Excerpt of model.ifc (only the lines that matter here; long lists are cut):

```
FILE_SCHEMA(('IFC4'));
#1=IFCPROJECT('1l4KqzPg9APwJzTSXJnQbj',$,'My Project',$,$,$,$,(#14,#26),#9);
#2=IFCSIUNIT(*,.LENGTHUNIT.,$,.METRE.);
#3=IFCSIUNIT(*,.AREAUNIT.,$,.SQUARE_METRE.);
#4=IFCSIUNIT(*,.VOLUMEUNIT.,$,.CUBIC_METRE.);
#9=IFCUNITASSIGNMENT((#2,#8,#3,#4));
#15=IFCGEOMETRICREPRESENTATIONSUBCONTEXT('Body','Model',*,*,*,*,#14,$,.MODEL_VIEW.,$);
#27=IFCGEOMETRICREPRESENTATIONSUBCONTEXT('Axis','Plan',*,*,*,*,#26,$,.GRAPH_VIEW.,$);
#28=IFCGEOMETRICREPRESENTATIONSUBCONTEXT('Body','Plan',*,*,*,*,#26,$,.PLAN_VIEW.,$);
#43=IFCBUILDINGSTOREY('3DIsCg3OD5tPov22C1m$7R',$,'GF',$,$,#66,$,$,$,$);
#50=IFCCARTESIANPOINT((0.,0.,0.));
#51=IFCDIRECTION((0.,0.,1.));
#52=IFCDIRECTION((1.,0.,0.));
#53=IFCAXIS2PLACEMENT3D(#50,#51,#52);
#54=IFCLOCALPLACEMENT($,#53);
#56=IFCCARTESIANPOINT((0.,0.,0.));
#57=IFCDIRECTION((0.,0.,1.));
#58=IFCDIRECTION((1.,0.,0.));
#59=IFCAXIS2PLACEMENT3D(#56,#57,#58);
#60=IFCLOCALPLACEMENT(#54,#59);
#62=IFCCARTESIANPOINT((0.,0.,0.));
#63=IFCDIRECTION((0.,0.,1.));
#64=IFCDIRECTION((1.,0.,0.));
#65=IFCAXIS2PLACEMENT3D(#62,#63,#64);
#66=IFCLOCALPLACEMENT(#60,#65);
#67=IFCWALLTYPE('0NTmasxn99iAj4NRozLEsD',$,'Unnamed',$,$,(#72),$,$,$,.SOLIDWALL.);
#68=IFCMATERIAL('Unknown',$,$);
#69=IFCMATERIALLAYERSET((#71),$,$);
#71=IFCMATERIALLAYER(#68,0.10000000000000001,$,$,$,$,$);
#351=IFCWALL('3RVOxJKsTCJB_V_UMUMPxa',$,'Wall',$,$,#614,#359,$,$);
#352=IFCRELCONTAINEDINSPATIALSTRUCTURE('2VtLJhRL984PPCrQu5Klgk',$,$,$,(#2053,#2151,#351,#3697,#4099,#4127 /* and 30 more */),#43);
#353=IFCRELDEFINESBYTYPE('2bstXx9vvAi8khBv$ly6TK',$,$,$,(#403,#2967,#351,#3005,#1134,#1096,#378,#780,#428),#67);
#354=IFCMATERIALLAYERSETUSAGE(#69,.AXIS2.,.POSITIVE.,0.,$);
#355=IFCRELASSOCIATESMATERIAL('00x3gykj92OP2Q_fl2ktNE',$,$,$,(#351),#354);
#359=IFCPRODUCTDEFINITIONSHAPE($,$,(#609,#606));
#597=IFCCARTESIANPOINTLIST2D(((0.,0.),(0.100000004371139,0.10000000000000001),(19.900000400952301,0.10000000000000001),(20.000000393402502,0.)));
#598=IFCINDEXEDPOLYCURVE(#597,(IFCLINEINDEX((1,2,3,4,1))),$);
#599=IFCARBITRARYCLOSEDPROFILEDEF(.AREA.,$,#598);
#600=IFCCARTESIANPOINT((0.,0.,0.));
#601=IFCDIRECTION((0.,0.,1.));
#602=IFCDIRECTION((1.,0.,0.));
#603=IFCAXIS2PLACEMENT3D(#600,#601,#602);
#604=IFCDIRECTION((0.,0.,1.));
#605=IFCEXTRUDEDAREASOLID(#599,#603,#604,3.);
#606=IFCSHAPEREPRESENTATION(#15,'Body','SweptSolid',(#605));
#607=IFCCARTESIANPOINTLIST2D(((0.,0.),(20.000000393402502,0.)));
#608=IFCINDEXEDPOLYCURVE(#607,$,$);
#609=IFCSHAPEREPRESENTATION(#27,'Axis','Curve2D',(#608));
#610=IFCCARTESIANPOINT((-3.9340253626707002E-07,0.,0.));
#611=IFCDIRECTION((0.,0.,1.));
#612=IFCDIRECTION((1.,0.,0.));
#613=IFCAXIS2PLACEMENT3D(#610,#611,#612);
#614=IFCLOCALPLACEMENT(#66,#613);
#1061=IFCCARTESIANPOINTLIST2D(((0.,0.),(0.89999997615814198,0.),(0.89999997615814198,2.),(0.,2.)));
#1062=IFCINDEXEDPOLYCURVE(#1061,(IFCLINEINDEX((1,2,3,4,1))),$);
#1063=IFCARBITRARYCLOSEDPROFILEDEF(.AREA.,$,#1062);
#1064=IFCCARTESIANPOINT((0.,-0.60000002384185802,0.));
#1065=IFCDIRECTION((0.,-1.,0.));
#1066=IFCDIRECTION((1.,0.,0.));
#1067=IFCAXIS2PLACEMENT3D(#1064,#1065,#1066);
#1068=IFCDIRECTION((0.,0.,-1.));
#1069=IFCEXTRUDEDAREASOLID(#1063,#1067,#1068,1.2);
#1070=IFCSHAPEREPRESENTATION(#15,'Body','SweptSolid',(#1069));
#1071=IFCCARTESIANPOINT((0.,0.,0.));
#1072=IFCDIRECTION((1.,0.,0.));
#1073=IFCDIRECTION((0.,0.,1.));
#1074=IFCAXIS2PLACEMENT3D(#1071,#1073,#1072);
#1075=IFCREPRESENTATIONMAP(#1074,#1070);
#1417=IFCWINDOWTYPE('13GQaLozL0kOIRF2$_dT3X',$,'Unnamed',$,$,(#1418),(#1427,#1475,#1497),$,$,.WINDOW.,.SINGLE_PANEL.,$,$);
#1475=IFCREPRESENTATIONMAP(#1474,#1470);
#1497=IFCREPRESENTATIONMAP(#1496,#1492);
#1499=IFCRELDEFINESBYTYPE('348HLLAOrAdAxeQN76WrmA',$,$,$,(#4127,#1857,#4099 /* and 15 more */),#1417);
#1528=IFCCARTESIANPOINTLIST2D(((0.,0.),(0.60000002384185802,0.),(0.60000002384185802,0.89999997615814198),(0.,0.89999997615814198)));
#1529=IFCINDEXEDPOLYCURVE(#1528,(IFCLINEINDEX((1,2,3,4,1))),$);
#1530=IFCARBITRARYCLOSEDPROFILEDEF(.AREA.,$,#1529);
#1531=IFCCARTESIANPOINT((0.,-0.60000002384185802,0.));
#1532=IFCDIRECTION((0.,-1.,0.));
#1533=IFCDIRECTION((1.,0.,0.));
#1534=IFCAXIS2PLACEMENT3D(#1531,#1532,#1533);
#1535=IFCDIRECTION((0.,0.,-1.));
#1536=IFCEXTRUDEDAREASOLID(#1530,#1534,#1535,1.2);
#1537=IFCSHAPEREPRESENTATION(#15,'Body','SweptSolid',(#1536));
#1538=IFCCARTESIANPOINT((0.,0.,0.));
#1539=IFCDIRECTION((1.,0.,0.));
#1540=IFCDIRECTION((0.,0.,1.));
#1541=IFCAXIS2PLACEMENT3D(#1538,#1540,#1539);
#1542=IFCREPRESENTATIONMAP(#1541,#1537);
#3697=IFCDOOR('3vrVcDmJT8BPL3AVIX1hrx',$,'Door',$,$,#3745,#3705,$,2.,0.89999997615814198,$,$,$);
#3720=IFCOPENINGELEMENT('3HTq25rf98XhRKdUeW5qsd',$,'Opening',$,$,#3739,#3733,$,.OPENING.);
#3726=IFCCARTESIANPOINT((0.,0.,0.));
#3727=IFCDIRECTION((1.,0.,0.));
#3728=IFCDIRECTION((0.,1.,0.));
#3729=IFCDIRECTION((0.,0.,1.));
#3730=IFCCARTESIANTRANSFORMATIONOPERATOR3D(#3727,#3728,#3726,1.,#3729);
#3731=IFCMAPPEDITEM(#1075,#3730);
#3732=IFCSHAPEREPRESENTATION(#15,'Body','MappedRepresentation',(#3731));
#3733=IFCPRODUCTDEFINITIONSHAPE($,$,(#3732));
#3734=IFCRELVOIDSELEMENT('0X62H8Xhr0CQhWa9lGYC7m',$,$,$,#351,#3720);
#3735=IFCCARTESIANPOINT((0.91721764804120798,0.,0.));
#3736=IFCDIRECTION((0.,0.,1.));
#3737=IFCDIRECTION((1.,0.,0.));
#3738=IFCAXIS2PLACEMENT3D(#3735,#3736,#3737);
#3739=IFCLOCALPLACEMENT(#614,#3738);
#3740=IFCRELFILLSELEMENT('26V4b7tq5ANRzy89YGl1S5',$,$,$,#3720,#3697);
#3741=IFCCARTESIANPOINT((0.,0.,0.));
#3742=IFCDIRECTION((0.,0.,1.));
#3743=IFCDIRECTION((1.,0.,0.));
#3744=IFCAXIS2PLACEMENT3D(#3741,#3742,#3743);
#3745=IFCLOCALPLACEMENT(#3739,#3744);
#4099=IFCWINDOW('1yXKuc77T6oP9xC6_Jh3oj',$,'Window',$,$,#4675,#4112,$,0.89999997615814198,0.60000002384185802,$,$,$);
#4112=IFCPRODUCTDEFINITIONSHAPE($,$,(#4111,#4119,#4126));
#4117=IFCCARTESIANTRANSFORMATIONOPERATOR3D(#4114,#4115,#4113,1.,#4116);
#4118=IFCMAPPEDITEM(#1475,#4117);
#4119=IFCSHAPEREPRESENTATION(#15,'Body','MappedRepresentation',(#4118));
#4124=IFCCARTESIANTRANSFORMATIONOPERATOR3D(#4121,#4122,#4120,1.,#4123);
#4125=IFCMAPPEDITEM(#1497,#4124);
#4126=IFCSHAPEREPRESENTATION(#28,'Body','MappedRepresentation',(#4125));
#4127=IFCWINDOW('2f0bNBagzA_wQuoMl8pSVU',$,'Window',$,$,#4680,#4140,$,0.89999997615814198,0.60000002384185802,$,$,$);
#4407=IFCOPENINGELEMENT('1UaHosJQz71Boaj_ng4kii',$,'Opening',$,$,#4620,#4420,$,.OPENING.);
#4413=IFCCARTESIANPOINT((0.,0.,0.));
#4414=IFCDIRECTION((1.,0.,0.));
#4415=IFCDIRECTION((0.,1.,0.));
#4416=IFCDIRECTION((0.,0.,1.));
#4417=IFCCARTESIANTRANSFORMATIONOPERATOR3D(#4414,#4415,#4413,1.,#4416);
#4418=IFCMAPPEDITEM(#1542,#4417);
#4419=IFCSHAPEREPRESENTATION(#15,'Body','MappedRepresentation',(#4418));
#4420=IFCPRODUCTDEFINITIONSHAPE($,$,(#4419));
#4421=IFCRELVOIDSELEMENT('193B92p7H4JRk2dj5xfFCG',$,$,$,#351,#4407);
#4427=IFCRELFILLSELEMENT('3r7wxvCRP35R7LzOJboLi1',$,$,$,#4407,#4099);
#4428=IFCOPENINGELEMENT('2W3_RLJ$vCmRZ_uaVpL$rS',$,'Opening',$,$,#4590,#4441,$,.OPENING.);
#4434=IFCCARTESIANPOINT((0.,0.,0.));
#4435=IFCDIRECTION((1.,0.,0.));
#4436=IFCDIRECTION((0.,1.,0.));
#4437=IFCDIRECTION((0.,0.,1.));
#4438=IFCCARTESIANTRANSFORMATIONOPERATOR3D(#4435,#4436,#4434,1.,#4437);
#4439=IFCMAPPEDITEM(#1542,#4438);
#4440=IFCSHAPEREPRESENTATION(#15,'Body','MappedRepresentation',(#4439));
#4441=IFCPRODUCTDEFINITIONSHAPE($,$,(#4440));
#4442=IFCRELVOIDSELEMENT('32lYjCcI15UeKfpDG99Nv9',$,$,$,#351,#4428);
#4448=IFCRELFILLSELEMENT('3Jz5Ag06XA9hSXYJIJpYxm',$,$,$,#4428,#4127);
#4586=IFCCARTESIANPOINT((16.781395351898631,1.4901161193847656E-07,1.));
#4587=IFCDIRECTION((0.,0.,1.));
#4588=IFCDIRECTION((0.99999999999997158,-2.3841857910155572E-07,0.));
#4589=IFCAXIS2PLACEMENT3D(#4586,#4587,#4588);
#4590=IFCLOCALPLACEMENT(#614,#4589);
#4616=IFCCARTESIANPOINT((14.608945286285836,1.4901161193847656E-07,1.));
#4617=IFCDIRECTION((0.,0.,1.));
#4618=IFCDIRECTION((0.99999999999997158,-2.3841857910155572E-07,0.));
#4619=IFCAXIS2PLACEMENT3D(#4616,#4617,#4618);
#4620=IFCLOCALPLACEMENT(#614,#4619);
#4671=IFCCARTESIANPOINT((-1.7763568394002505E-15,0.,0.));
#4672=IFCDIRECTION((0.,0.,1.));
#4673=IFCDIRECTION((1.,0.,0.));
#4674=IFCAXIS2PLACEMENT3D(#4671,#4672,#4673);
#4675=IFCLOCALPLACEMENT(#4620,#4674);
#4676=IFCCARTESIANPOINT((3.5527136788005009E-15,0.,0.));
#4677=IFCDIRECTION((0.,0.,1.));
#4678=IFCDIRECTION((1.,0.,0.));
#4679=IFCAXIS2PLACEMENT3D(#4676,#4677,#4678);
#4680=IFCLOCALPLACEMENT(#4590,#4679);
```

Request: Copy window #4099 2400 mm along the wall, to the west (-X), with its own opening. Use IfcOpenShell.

```python
import ifcopenshell
import ifcopenshell.api.feature
import ifcopenshell.api.geometry
import ifcopenshell.api.root
import ifcopenshell.geom
import ifcopenshell.util.element
import ifcopenshell.util.placement
import ifcopenshell.util.shape
import ifcopenshell.util.unit

model = ifcopenshell.open("model.ifc")
unit_scale = ifcopenshell.util.unit.calculate_unit_scale(model)
settings = ifcopenshell.geom.settings()


def volume(element):
    """Net volume in cubic metres, openings subtracted."""
    shape = ifcopenshell.geom.create_shape(settings, element)
    return ifcopenshell.util.shape.get_volume(shape.geometry)


window = model.by_guid("1yXKuc77T6oP9xC6_Jh3oj")
opening = window.FillsVoids[0].RelatingOpeningElement
wall = opening.VoidsElements[0].RelatingBuildingElement
before = volume(wall)
shift = ifcopenshell.util.placement.get_local_placement(wall.ObjectPlacement)[:3, 0] * -2.4 / unit_scale

# copy_class copies the void relationship, type, container and properties, but no geometry.
new_opening = ifcopenshell.api.root.copy_class(model, product=opening)
new_opening.Representation = ifcopenshell.util.element.copy_deep(
    model, opening.Representation, exclude=["IfcGeometricRepresentationContext", "IfcRepresentationMap"]
)
new_window = ifcopenshell.api.root.copy_class(model, product=window)
new_window.Representation = ifcopenshell.util.element.copy_deep(
    model, window.Representation, exclude=["IfcGeometricRepresentationContext", "IfcRepresentationMap"]
)
ifcopenshell.api.feature.add_filling(model, opening=new_opening, element=new_window)

for old, new in ((opening, new_opening), (window, new_window)):
    matrix = ifcopenshell.util.placement.get_local_placement(old.ObjectPlacement)
    matrix[:3, 3] += shift
    ifcopenshell.api.geometry.edit_object_placement(model, product=new, matrix=matrix, is_si=False)

after = volume(wall)

print(f"wall volume {before:.3f} -> {after:.3f} m3")

model.write("model_v2.ifc")
```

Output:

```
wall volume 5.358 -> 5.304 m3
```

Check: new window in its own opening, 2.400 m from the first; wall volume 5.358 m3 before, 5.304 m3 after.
